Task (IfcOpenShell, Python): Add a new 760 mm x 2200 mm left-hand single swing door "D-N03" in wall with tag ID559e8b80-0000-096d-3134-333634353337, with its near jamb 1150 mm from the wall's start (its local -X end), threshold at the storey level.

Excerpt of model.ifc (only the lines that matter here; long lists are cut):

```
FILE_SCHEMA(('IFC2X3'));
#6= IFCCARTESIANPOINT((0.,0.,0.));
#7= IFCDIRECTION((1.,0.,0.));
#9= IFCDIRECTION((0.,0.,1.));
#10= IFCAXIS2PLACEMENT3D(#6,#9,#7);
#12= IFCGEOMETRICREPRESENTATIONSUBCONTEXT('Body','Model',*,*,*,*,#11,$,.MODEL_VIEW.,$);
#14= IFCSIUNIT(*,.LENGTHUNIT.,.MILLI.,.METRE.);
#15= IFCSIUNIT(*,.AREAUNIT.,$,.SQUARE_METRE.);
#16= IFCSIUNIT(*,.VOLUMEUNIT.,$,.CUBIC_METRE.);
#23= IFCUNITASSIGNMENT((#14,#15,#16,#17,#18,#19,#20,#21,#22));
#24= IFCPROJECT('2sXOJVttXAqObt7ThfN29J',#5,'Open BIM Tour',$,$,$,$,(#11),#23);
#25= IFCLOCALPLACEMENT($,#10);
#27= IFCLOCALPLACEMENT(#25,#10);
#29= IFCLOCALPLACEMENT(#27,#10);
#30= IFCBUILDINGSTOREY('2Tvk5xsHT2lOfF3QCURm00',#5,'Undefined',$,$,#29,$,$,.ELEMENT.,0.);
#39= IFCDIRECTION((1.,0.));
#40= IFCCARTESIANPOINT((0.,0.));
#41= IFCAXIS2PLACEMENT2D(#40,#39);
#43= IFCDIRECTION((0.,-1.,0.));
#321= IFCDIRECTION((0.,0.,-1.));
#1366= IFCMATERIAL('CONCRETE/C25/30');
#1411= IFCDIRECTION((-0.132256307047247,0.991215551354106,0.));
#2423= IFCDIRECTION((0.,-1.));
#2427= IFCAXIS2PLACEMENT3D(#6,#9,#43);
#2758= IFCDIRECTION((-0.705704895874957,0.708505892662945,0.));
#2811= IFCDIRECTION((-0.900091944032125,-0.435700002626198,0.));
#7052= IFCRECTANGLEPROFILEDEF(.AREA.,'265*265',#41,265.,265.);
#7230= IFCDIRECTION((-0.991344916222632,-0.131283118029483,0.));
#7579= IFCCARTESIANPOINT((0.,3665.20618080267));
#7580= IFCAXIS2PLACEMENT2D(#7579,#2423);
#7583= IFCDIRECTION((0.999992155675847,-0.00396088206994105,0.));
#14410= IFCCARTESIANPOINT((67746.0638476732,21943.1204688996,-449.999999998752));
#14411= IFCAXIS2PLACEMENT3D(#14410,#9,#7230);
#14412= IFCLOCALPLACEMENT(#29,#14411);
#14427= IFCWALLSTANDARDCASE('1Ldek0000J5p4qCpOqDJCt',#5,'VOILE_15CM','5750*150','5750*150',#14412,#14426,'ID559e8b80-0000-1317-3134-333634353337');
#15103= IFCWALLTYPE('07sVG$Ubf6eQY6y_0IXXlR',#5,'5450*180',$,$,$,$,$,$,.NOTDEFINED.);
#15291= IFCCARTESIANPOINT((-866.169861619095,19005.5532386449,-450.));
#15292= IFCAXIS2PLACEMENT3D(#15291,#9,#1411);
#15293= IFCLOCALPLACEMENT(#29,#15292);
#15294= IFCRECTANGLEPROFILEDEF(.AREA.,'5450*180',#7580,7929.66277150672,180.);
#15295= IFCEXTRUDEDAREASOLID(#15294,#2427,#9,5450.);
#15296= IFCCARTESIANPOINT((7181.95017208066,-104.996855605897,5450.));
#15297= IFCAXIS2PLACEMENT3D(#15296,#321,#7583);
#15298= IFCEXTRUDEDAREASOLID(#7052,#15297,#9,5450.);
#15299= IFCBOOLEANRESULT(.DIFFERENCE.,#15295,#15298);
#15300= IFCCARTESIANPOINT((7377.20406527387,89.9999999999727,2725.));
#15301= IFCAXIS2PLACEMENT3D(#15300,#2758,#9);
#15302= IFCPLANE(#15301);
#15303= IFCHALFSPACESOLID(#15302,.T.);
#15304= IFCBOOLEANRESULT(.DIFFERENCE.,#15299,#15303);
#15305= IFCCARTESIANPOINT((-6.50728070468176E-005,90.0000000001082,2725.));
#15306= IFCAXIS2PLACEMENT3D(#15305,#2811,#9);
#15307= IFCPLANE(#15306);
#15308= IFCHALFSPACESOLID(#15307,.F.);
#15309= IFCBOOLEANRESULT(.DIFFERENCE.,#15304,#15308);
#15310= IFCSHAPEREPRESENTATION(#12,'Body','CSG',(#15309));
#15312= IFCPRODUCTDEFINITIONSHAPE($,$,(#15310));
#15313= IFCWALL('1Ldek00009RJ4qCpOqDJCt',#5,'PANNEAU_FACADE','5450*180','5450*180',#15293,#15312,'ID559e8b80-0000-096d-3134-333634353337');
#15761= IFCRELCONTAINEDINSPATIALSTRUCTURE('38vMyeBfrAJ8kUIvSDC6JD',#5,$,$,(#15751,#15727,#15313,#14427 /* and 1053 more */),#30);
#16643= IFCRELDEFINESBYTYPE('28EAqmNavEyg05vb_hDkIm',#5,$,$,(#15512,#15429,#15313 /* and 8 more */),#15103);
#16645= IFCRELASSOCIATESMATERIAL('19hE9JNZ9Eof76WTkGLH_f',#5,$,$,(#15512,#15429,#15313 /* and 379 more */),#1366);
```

```python
import numpy as np
import ifcopenshell
import ifcopenshell.api.feature
import ifcopenshell.api.geometry
import ifcopenshell.api.root
import ifcopenshell.api.spatial
import ifcopenshell.api.type
import ifcopenshell.geom
import ifcopenshell.util.element
import ifcopenshell.util.placement
import ifcopenshell.util.representation
import ifcopenshell.util.shape
import ifcopenshell.util.unit

model = ifcopenshell.open("model.ifc")
unit_scale = ifcopenshell.util.unit.calculate_unit_scale(model)
settings = ifcopenshell.geom.settings()


def volume(element):
    """Net volume in cubic metres, openings subtracted."""
    shape = ifcopenshell.geom.create_shape(settings, element)
    return ifcopenshell.util.shape.get_volume(shape.geometry)


wall = model.by_id(15313)
storey = ifcopenshell.util.element.get_container(wall, ifc_class="IfcBuildingStorey")
context = ifcopenshell.util.representation.get_context(model, "Model", "Body", "MODEL_VIEW")
before = volume(wall)

width, height, from_end, sill = 0.76, 2.2, 1.15, 0.0  # metres

# The wall runs along its own X axis, and the end named is its -X end.
wall_shape = ifcopenshell.geom.create_shape(settings, wall)
x, y, z = ifcopenshell.util.shape.get_vertices(wall_shape.geometry).T
start = x.min() + from_end
face, thickness = float(y.min()), float(y.max() - y.min())
wall_matrix = ifcopenshell.util.placement.get_local_placement(wall.ObjectPlacement)
level = ifcopenshell.util.placement.get_local_placement(storey.ObjectPlacement)[2, 3]


def in_wall(x, y):
    """Placement at x, y metres in the wall's axes, at sill height."""
    matrix = wall_matrix.copy()
    matrix[:, 3] = wall_matrix @ np.array([x / unit_scale, y / unit_scale, 0.0, 1.0])
    matrix[2, 3] = level + sill / unit_scale
    return matrix


# Opening: a box that overshoots both wall faces by 50 mm.
opening = ifcopenshell.api.root.create_entity(model, ifc_class="IfcOpeningElement")
box = ifcopenshell.api.geometry.add_wall_representation(
    model, context=context, length=width, height=height, thickness=thickness + 0.1
)
ifcopenshell.api.geometry.assign_representation(model, product=opening, representation=box)
ifcopenshell.api.geometry.edit_object_placement(model, product=opening, matrix=in_wall(start, face - 0.05), is_si=False)
ifcopenshell.api.feature.add_feature(model, feature=opening, element=wall)

door = ifcopenshell.api.root.create_entity(model, ifc_class="IfcDoor", name="D-N03")
door.OverallWidth, door.OverallHeight = width / unit_scale, height / unit_scale
body = ifcopenshell.api.geometry.add_door_representation(
    model,
    context=context,
    overall_width=door.OverallWidth,
    overall_height=door.OverallHeight,
    operation_type="SINGLE_SWING_LEFT",
    lining_properties={"LiningDepth": thickness / unit_scale, "ThresholdDepth": thickness / unit_scale},
)
ifcopenshell.api.geometry.assign_representation(model, product=door, representation=body)
ifcopenshell.api.spatial.assign_container(model, products=[door], relating_structure=storey)
fills = ifcopenshell.api.feature.add_filling(model, opening=opening, element=door)
fills.OwnerHistory = door.OwnerHistory  # required in IFC2X3

# IFC2X3 keeps the operation on the door style.
style = ifcopenshell.api.root.create_entity(model, ifc_class="IfcDoorStyle", name="D-N03")
style.OperationType, style.ConstructionType = "SINGLE_SWING_LEFT", "NOTDEFINED"
style.ParameterTakesPrecedence = style.Sizeable = False
ifcopenshell.api.type.assign_type(model, related_objects=[door], relating_type=style)

# The lining spans the wall, so the door starts at the wall face.
ifcopenshell.api.geometry.edit_object_placement(model, product=door, matrix=in_wall(start, face), is_si=False)

after = volume(wall)

print(f"wall volume {before:.3f} -> {after:.3f} m3")

model.write("model-out.ifc")
```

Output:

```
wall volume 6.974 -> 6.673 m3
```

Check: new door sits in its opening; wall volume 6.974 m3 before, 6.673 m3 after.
